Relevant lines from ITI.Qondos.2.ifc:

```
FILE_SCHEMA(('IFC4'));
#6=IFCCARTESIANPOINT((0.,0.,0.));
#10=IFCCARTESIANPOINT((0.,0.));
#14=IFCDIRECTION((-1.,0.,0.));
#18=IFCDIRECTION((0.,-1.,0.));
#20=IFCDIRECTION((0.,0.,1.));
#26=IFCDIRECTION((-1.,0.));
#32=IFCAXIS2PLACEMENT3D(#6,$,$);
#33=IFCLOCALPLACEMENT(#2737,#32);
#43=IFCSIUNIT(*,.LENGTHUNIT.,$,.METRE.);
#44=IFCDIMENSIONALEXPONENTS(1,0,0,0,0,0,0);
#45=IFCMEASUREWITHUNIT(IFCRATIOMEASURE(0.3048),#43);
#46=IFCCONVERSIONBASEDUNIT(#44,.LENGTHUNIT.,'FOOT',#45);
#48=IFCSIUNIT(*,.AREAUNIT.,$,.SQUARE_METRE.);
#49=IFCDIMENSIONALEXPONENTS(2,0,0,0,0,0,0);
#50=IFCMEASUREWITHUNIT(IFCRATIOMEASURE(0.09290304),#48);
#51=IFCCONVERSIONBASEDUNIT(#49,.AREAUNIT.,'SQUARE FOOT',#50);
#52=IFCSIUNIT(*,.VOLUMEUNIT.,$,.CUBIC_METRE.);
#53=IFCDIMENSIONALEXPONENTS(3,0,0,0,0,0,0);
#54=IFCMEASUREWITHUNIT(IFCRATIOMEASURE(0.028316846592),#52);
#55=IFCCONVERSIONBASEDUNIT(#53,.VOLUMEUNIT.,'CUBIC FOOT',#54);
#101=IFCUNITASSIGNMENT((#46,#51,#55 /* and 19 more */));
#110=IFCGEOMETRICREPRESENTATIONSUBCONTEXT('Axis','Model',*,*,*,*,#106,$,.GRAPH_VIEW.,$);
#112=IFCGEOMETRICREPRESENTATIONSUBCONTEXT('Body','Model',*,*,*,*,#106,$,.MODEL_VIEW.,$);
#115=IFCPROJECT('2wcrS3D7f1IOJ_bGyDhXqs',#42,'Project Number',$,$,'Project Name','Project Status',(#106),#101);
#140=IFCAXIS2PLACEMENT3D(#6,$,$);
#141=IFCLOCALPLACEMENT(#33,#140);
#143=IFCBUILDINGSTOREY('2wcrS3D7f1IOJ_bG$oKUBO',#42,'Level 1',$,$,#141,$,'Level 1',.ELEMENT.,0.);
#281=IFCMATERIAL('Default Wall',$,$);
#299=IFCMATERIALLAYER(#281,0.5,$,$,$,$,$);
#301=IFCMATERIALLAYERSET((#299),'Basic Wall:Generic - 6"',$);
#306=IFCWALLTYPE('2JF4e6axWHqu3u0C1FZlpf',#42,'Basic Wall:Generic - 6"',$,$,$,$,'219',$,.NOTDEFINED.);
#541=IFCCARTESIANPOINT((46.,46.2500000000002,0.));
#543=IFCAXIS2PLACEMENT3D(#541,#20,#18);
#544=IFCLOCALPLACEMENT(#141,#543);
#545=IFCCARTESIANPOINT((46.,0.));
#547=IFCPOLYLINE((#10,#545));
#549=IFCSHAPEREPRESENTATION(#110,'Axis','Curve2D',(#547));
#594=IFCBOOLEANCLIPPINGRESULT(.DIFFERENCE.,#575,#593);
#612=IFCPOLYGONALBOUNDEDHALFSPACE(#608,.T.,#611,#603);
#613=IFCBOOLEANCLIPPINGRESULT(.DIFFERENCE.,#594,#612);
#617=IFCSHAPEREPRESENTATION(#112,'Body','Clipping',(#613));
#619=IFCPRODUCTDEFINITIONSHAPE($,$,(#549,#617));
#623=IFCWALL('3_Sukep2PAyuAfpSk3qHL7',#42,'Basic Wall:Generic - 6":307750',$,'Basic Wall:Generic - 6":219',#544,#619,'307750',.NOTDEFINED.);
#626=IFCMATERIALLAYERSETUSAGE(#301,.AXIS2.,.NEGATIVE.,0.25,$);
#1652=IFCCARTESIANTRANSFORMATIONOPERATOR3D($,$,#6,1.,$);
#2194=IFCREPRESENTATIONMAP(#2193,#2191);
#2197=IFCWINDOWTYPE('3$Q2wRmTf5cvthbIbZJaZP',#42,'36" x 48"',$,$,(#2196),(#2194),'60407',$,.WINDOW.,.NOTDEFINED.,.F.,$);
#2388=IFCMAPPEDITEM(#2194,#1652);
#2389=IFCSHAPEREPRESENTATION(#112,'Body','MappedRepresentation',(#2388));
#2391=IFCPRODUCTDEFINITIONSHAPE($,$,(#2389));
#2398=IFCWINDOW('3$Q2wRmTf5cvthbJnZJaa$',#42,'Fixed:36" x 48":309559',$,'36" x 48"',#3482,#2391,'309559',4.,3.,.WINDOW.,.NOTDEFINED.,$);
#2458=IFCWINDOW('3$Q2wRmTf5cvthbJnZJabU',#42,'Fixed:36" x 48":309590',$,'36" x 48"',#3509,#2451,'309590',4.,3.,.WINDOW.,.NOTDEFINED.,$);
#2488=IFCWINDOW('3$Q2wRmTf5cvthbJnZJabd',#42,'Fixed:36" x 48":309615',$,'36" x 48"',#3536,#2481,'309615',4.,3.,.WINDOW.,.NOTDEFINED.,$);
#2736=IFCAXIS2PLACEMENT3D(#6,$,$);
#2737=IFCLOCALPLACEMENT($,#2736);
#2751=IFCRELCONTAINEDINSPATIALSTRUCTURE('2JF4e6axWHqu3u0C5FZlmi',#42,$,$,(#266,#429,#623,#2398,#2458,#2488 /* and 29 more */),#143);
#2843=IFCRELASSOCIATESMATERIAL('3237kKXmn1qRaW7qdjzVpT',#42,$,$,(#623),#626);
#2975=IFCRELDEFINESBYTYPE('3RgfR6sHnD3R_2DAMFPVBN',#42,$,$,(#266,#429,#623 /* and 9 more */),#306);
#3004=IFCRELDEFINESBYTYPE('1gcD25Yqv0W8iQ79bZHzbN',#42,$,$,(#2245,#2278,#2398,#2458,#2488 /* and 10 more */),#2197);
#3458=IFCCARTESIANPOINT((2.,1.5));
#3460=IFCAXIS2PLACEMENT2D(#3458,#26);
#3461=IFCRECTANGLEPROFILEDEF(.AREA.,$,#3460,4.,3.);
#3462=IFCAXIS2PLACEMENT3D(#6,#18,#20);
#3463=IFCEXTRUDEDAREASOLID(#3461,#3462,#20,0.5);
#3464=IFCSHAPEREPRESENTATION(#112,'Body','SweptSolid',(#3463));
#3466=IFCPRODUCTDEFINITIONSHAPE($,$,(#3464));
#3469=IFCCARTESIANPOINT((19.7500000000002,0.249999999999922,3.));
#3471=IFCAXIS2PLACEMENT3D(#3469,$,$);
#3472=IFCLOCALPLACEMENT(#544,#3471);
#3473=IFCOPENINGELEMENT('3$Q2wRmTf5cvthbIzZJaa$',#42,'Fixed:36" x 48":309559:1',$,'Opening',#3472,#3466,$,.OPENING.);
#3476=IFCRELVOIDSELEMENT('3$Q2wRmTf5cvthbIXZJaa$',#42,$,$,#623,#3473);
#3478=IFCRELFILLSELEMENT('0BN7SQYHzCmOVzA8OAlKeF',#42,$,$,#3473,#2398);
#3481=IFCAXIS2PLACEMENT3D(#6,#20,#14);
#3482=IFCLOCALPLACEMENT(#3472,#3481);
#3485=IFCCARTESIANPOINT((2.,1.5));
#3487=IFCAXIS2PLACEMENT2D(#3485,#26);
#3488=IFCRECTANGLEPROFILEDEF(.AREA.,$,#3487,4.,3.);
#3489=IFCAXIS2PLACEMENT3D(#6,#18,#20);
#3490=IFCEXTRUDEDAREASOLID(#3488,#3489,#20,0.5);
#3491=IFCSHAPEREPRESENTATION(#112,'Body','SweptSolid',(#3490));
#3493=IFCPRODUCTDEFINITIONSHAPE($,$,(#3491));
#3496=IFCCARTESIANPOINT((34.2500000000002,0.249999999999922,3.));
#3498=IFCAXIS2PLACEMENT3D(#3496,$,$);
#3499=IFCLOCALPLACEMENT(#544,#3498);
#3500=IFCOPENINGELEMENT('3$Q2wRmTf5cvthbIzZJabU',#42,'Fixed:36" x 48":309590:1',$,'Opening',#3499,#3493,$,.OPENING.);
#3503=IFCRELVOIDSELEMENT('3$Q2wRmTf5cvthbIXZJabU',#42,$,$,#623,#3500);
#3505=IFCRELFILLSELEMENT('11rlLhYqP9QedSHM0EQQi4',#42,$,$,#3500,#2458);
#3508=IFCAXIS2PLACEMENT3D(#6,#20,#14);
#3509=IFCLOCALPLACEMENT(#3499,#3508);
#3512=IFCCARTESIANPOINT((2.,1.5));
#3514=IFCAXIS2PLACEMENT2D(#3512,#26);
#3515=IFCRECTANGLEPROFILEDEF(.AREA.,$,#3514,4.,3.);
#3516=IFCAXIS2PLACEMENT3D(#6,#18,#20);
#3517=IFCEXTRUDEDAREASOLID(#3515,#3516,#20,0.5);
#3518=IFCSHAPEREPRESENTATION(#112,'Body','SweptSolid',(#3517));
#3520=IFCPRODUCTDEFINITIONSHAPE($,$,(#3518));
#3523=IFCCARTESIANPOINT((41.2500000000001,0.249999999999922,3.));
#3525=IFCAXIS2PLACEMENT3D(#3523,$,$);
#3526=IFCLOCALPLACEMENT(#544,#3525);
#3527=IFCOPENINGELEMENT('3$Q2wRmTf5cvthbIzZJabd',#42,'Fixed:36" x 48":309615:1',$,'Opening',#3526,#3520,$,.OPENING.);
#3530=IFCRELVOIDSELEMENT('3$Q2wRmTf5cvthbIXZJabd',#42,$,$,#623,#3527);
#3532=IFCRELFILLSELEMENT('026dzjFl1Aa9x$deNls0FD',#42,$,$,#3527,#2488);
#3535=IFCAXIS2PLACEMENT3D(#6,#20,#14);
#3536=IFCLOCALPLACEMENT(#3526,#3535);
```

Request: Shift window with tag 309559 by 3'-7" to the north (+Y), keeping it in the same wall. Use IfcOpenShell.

```python
import ifcopenshell
import ifcopenshell.api.geometry
import ifcopenshell.util.placement
import ifcopenshell.util.unit

model = ifcopenshell.open("ITI.Qondos.2.ifc")
unit_scale = ifcopenshell.util.unit.calculate_unit_scale(model)

window = model.by_guid("3$Q2wRmTf5cvthbJnZJaa$")
opening = window.FillsVoids[0].RelatingOpeningElement
wall = opening.VoidsElements[0].RelatingBuildingElement

wall_matrix = ifcopenshell.util.placement.get_local_placement(wall.ObjectPlacement)
shift = wall_matrix[:3, 0] * -43 * 0.0254 / unit_scale
before = ifcopenshell.util.placement.get_local_placement(window.ObjectPlacement)[:3, 3].copy()

# The window is placed relative to its opening, so it follows when the opening moves.
matrix = ifcopenshell.util.placement.get_local_placement(opening.ObjectPlacement)
matrix[:3, 3] += shift
ifcopenshell.api.geometry.edit_object_placement(
    model, product=opening, matrix=matrix, is_si=False, should_transform_children=True
)

after = ifcopenshell.util.placement.get_local_placement(window.ObjectPlacement)[:3, 3]
print("window moved by", (after - before).round(3) + 0.0)

model.write("ITI.Qondos.2-out.ifc")
```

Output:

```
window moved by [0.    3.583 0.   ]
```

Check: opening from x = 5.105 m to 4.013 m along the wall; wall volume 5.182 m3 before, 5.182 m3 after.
